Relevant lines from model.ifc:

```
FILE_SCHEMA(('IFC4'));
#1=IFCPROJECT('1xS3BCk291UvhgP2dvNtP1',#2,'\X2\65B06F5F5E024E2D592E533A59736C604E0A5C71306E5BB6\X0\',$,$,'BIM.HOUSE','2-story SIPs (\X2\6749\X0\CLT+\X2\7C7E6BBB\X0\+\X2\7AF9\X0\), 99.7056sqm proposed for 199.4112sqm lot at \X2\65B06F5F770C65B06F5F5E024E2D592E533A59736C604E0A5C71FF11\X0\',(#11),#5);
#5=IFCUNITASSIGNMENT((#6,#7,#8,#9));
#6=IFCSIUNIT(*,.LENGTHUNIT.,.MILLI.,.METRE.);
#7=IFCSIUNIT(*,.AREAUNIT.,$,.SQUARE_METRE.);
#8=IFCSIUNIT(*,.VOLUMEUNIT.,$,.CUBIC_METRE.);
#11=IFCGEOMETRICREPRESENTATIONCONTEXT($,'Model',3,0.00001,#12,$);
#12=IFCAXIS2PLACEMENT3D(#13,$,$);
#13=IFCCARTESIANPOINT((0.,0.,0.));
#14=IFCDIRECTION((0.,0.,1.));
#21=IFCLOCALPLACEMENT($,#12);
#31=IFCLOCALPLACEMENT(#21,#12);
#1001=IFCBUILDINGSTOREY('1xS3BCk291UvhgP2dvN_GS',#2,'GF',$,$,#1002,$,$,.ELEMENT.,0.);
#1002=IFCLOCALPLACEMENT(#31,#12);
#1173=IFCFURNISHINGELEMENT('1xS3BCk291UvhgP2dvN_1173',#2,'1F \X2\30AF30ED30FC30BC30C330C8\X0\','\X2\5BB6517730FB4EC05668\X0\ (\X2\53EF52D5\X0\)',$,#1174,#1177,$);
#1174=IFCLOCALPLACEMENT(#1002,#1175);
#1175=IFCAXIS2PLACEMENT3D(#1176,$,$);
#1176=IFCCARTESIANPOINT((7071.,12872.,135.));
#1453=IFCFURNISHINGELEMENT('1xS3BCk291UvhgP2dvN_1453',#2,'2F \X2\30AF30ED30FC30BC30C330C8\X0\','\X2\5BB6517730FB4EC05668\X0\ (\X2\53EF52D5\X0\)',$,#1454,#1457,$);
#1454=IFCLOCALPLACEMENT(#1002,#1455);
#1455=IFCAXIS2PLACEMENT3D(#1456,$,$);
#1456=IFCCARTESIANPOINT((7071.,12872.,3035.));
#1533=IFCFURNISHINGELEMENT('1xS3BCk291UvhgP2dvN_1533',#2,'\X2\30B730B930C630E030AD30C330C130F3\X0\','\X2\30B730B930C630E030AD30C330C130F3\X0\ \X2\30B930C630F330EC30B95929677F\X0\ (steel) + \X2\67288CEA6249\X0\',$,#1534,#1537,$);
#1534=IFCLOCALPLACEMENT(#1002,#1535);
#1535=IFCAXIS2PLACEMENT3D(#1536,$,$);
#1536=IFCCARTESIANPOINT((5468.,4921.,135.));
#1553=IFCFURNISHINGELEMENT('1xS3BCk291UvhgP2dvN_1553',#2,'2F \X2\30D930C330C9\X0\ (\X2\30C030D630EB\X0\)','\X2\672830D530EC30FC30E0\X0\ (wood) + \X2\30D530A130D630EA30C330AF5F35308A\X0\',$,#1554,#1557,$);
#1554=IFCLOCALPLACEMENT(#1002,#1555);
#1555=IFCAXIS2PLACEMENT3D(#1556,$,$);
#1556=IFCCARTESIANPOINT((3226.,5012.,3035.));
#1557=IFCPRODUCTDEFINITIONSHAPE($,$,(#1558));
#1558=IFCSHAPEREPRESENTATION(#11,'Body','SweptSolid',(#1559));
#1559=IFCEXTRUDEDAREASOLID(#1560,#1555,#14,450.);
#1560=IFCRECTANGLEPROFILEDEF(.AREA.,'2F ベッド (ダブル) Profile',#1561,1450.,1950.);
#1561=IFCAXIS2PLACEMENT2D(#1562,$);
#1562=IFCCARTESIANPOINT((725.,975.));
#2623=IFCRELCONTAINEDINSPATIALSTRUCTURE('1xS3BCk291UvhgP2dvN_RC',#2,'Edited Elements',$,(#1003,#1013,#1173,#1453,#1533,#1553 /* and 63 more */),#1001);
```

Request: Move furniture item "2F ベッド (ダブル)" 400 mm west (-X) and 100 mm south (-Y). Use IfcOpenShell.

```python
import ifcopenshell
import ifcopenshell.api.geometry
import ifcopenshell.util.placement

model = ifcopenshell.open("model.ifc")

item = model.by_guid("1xS3BCk291UvhgP2dvN_1553")
matrix = ifcopenshell.util.placement.get_local_placement(item.ObjectPlacement)
matrix[0, 3] -= 400.0
matrix[1, 3] -= 100.0
ifcopenshell.api.geometry.edit_object_placement(model, product=item, matrix=matrix, is_si=False)

print(ifcopenshell.util.placement.get_local_placement(item.ObjectPlacement).round(3) + 0.0)

model.write("model_v2.ifc")
```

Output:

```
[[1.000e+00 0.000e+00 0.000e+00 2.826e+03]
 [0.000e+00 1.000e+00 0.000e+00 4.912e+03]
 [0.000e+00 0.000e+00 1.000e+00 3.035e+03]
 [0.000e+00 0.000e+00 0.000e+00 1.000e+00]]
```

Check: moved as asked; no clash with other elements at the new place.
